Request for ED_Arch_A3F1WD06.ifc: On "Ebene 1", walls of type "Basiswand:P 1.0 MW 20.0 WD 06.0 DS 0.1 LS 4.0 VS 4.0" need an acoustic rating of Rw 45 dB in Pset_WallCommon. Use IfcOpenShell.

First a look at what the model holds.

```python
import ifcopenshell
import ifcopenshell.util.element

model = ifcopenshell.open("ED_Arch_A3F1WD06.ifc")
print(model.schema)
storey = next(s for s in model.by_type("IfcBuildingStorey") if s.Name == "Ebene 1")
walls = [e for e in ifcopenshell.util.element.get_decomposition(storey) if e.is_a("IfcWall")]
seen = {}
for e in walls:
    element_type = ifcopenshell.util.element.get_type(e)
    key = (element_type.Name if element_type != e and element_type else None, ifcopenshell.util.element.get_pset(e, "Pset_WallCommon", "AcousticRating"))
    seen[key] = seen.get(key, 0) + 1
for (name, value), count in sorted(seen.items(), key=str):
    print(count, "x", name, "|", value)
```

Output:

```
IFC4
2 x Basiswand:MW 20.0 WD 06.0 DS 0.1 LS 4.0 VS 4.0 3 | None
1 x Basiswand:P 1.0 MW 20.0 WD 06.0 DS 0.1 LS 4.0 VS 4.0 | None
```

```python
import ifcopenshell
import ifcopenshell.api.pset
import ifcopenshell.util.element

model = ifcopenshell.open("ED_Arch_A3F1WD06.ifc")

storey = next(s for s in model.by_type("IfcBuildingStorey") if s.Name == "Ebene 1")
walls = [e for e in ifcopenshell.util.element.get_decomposition(storey) if e.is_a("IfcWall")]

count = 0
for e in walls:
    element_type = ifcopenshell.util.element.get_type(e)
    if element_type in (None, e) or element_type.Name != "Basiswand:P 1.0 MW 20.0 WD 06.0 DS 0.1 LS 4.0 VS 4.0":
        continue
    # add_pset returns the element's existing set when there is one.
    pset = ifcopenshell.api.pset.add_pset(model, product=e, name="Pset_WallCommon")
    ifcopenshell.api.pset.edit_pset(model, pset=pset, properties={"AcousticRating": "Rw 45 dB"})
    count += 1

print(count, "walls updated")

model.write("ED_Arch_A3F1WD06-out.ifc")
```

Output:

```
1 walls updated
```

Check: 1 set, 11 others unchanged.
